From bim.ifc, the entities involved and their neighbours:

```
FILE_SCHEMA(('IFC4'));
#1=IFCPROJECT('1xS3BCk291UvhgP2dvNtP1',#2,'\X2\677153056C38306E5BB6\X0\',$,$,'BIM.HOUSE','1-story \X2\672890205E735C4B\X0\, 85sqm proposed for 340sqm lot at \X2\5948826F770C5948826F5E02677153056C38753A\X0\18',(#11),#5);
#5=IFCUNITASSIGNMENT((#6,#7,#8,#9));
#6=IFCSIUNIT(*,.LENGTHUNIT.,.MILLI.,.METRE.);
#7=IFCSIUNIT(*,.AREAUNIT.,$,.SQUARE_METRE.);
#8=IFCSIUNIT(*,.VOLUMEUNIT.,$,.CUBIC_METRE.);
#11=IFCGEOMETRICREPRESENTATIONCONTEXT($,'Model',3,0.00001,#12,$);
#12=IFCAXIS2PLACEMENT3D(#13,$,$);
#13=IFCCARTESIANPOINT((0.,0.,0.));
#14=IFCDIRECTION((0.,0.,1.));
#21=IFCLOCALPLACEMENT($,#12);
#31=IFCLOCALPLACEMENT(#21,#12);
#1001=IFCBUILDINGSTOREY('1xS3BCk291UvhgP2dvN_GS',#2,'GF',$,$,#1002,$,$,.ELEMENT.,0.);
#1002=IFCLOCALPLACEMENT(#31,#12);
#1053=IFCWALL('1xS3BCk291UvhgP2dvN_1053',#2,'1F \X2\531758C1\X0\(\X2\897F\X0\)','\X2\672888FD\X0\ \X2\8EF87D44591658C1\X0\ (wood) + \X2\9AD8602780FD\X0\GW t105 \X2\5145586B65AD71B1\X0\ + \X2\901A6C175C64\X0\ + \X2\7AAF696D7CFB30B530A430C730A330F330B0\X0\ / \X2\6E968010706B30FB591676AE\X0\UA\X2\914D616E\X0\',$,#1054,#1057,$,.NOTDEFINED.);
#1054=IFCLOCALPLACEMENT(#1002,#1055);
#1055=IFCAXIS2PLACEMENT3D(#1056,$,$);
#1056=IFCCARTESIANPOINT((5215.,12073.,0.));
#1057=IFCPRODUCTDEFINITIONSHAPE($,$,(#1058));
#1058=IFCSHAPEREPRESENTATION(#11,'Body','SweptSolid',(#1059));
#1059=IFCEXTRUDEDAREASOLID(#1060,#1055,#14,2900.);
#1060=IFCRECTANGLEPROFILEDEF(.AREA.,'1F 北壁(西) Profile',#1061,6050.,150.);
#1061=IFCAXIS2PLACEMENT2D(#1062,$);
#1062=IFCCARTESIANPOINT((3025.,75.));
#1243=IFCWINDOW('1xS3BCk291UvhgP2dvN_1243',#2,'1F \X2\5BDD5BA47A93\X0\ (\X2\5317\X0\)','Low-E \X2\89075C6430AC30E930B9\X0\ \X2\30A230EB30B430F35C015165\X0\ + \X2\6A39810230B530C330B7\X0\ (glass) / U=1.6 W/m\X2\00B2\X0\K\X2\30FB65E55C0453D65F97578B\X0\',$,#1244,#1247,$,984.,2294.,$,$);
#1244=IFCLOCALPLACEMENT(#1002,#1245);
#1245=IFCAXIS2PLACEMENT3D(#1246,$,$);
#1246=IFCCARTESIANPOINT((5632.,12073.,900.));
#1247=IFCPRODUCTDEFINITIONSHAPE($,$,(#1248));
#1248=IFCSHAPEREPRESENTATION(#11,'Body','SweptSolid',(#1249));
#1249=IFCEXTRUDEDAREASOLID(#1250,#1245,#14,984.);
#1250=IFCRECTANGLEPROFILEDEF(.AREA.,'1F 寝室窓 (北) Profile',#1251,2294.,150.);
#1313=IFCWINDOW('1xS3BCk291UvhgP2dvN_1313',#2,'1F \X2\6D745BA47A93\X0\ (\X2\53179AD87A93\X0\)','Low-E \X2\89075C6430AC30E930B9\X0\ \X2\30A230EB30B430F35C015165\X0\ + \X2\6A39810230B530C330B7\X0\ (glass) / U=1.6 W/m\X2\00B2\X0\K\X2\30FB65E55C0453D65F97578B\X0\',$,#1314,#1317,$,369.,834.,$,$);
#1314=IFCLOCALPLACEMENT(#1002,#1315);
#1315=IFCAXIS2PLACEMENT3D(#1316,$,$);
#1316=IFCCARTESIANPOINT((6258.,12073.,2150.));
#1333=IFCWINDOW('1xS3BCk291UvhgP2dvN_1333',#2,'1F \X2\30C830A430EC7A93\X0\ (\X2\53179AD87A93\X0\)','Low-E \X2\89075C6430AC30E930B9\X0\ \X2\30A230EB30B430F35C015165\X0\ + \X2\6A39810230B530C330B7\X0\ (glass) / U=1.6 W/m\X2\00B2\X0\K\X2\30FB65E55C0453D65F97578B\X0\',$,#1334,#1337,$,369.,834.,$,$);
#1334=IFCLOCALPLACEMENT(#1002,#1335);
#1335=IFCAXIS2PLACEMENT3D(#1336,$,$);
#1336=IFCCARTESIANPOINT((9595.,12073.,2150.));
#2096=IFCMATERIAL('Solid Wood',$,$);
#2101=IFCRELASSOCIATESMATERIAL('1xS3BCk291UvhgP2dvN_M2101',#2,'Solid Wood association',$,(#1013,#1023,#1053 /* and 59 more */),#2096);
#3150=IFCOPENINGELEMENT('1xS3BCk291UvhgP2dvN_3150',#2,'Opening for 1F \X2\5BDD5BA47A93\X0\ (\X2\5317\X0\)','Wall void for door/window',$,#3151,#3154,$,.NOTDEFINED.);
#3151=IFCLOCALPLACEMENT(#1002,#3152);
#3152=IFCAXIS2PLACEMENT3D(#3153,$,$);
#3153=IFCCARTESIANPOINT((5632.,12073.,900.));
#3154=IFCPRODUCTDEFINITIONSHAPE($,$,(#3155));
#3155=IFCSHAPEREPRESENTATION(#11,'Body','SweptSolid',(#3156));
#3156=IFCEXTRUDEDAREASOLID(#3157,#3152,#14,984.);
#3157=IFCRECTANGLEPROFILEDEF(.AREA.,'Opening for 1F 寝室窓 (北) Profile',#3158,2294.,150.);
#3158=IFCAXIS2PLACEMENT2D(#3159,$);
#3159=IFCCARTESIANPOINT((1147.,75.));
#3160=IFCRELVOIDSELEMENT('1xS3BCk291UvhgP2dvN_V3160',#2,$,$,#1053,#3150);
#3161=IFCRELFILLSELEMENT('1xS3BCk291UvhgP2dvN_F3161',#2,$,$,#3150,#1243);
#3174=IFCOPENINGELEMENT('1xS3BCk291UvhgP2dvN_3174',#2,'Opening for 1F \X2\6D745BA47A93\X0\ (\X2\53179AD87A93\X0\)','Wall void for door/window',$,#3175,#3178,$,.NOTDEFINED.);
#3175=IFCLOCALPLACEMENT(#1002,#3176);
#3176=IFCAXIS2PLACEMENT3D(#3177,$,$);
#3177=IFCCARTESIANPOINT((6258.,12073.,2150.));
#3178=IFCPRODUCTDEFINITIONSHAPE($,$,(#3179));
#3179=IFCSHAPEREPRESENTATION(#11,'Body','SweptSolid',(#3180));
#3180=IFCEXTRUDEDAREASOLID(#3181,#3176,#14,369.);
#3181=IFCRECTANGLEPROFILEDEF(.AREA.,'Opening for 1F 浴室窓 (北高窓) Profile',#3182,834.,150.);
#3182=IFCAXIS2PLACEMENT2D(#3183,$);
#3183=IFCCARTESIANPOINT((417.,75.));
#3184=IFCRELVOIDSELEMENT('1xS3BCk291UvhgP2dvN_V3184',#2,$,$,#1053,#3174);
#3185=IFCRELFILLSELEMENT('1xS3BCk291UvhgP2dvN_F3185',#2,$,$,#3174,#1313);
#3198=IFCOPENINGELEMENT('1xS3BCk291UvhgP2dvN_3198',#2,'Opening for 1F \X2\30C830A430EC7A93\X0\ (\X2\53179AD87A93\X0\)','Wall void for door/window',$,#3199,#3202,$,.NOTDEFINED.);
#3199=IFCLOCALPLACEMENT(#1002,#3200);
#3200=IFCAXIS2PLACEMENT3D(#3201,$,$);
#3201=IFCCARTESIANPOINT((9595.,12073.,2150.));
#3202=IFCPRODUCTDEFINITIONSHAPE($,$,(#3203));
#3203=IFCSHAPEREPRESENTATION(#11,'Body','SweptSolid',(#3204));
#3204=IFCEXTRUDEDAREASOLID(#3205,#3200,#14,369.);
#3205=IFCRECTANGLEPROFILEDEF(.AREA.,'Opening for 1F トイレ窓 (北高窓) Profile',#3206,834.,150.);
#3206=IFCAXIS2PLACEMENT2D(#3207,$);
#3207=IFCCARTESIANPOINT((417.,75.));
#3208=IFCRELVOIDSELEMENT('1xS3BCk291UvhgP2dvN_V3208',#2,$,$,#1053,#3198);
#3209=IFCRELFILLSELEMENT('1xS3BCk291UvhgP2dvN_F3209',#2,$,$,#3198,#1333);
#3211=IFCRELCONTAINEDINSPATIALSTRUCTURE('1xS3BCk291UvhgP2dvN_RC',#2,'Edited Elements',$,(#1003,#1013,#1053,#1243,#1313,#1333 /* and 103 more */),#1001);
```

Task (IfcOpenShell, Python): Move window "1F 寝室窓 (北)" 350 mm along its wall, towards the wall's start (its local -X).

```python
import ifcopenshell
import ifcopenshell.api.geometry
import ifcopenshell.util.placement
import ifcopenshell.util.unit

model = ifcopenshell.open("bim.ifc")
unit_scale = ifcopenshell.util.unit.calculate_unit_scale(model)

window = model.by_guid("1xS3BCk291UvhgP2dvN_1243")
opening = window.FillsVoids[0].RelatingOpeningElement
wall = opening.VoidsElements[0].RelatingBuildingElement

wall_matrix = ifcopenshell.util.placement.get_local_placement(wall.ObjectPlacement)
shift = wall_matrix[:3, 0] * -0.35 / unit_scale
before = ifcopenshell.util.placement.get_local_placement(window.ObjectPlacement)[:3, 3].copy()

# The window is not placed relative to its opening, so move both.
for product in (opening, window):
    matrix = ifcopenshell.util.placement.get_local_placement(product.ObjectPlacement)
    matrix[:3, 3] += shift
    ifcopenshell.api.geometry.edit_object_placement(model, product=product, matrix=matrix, is_si=False)

after = ifcopenshell.util.placement.get_local_placement(window.ObjectPlacement)[:3, 3]
print("window moved by", (after - before).round(3) + 0.0)

model.write("bim_edited.ifc")
```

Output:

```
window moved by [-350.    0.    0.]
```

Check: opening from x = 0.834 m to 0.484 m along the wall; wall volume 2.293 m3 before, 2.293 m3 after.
